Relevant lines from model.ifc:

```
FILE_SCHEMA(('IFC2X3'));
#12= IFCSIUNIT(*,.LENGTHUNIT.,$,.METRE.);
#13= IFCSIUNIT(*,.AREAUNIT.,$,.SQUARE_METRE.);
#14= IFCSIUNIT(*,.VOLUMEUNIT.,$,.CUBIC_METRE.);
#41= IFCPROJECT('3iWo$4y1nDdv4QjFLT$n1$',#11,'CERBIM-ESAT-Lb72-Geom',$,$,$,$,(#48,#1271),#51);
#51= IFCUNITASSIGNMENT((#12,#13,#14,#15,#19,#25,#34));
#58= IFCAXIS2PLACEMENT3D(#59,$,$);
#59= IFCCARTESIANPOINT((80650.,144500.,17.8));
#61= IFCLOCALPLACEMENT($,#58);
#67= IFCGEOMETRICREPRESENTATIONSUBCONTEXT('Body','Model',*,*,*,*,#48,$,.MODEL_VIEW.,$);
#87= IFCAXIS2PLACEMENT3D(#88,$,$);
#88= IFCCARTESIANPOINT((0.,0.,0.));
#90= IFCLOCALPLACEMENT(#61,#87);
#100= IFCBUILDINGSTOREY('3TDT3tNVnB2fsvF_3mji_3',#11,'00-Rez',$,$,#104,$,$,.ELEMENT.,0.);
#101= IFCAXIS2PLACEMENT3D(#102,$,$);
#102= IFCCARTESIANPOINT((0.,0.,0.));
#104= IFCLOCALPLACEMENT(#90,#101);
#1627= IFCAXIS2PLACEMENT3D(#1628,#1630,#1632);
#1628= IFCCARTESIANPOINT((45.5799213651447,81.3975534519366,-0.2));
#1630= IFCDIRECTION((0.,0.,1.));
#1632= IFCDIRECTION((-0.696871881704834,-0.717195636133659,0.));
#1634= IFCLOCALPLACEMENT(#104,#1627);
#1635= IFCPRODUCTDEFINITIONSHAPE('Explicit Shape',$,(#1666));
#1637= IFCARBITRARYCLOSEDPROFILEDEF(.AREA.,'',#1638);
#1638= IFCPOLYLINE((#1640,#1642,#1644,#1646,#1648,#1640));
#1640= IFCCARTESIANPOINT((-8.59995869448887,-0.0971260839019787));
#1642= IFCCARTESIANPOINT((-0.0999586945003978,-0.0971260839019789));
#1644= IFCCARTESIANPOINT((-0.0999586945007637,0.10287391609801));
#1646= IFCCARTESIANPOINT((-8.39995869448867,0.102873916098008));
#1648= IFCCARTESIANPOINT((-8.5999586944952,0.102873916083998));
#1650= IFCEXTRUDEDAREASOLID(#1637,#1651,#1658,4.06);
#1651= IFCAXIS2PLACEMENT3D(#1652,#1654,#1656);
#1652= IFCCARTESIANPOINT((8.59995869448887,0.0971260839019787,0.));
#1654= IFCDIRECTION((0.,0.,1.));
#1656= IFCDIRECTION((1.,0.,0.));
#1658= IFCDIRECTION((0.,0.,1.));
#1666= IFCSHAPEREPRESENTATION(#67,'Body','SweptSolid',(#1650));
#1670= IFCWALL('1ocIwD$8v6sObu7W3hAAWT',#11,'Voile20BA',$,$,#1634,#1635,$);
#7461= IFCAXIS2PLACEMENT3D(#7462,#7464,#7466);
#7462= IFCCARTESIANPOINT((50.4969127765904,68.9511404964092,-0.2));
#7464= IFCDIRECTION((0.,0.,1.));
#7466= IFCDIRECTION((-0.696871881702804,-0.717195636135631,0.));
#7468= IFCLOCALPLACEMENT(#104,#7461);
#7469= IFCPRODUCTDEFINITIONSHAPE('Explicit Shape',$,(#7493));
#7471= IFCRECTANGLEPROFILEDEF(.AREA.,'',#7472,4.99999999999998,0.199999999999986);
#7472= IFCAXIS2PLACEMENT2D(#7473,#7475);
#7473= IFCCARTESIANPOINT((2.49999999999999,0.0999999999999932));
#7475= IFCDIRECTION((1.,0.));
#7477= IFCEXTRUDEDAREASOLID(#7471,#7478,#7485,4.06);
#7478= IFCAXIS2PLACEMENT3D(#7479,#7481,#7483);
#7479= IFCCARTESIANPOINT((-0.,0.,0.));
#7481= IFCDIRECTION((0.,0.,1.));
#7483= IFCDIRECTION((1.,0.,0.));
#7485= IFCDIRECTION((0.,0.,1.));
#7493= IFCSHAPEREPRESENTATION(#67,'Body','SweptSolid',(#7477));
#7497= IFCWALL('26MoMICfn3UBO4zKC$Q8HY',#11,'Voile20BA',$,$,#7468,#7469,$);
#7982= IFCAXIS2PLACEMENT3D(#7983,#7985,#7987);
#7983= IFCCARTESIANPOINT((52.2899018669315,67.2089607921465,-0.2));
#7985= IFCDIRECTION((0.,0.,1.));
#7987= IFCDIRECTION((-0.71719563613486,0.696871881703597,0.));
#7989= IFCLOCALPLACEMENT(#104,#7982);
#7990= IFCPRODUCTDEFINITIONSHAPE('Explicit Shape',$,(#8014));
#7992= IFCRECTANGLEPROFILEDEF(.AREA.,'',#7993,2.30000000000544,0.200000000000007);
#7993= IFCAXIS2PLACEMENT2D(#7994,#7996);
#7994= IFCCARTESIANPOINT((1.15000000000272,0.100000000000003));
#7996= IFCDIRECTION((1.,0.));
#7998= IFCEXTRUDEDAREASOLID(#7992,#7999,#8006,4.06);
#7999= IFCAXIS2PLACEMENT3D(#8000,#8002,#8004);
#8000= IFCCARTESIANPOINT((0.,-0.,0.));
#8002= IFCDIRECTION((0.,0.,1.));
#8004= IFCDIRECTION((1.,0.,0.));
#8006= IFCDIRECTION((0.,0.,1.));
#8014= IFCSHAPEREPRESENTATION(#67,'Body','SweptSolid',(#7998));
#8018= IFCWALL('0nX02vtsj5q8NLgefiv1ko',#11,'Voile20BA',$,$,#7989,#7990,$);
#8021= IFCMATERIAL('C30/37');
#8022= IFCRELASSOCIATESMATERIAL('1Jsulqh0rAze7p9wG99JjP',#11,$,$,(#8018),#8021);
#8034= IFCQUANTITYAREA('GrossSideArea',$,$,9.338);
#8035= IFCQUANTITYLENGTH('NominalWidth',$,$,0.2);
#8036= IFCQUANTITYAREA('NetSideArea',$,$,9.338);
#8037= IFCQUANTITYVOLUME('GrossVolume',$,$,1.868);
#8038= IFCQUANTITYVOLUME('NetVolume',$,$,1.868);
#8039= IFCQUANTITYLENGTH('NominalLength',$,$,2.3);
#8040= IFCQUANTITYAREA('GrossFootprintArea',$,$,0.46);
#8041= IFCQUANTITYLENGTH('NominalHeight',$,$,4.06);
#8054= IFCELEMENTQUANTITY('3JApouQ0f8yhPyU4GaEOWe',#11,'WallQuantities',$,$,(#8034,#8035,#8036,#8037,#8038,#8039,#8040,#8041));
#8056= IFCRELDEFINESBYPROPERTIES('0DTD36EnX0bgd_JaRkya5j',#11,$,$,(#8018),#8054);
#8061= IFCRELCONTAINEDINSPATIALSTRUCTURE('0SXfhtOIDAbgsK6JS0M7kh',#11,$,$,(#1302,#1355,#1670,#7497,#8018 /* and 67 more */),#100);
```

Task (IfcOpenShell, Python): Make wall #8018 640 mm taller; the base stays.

```python
import ifcopenshell
import ifcopenshell.api.pset
import ifcopenshell.geom
import ifcopenshell.util.element
import ifcopenshell.util.representation
import ifcopenshell.util.shape
import ifcopenshell.util.unit

model = ifcopenshell.open("model.ifc")
unit_scale = ifcopenshell.util.unit.calculate_unit_scale(model)
area_scale = ifcopenshell.util.unit.calculate_unit_scale(model, "AREAUNIT")
volume_scale = ifcopenshell.util.unit.calculate_unit_scale(model, "VOLUMEUNIT")
settings = ifcopenshell.geom.settings()


def volume(element):
    """Net volume in cubic metres, openings subtracted."""
    shape = ifcopenshell.geom.create_shape(settings, element)
    return ifcopenshell.util.shape.get_volume(shape.geometry)


wall = model.by_id(8018)
before = volume(wall)

body = ifcopenshell.util.representation.get_representation(wall, "Model", "Body")
solid = body.Items[0]
old_height = solid.Depth
solid.Depth += 0.64
after = volume(wall)
thickness = 0.2  # wall thickness in metres

# Update the stored height, areas and volumes.
qto = model.by_id(ifcopenshell.util.element.get_pset(wall, "WallQuantities", should_inherit=False)["id"])
ifcopenshell.api.pset.edit_qto(model, qto=qto, properties={
    "GrossSideArea": ifcopenshell.util.element.get_pset(wall, "WallQuantities", "GrossSideArea") * solid.Depth / old_height,
    "NetSideArea": after / thickness / area_scale,
    "GrossVolume": ifcopenshell.util.element.get_pset(wall, "WallQuantities", "GrossVolume") * solid.Depth / old_height,
    "NetVolume": after / volume_scale,
    "NominalHeight": solid.Depth,
})

print(f"height {old_height:g} -> {solid.Depth:g}, volume {before:.3f} -> {after:.3f} m3")

model.write("model_v2.ifc")
```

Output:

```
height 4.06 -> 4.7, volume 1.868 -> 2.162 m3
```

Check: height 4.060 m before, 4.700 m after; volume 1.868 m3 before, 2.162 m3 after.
